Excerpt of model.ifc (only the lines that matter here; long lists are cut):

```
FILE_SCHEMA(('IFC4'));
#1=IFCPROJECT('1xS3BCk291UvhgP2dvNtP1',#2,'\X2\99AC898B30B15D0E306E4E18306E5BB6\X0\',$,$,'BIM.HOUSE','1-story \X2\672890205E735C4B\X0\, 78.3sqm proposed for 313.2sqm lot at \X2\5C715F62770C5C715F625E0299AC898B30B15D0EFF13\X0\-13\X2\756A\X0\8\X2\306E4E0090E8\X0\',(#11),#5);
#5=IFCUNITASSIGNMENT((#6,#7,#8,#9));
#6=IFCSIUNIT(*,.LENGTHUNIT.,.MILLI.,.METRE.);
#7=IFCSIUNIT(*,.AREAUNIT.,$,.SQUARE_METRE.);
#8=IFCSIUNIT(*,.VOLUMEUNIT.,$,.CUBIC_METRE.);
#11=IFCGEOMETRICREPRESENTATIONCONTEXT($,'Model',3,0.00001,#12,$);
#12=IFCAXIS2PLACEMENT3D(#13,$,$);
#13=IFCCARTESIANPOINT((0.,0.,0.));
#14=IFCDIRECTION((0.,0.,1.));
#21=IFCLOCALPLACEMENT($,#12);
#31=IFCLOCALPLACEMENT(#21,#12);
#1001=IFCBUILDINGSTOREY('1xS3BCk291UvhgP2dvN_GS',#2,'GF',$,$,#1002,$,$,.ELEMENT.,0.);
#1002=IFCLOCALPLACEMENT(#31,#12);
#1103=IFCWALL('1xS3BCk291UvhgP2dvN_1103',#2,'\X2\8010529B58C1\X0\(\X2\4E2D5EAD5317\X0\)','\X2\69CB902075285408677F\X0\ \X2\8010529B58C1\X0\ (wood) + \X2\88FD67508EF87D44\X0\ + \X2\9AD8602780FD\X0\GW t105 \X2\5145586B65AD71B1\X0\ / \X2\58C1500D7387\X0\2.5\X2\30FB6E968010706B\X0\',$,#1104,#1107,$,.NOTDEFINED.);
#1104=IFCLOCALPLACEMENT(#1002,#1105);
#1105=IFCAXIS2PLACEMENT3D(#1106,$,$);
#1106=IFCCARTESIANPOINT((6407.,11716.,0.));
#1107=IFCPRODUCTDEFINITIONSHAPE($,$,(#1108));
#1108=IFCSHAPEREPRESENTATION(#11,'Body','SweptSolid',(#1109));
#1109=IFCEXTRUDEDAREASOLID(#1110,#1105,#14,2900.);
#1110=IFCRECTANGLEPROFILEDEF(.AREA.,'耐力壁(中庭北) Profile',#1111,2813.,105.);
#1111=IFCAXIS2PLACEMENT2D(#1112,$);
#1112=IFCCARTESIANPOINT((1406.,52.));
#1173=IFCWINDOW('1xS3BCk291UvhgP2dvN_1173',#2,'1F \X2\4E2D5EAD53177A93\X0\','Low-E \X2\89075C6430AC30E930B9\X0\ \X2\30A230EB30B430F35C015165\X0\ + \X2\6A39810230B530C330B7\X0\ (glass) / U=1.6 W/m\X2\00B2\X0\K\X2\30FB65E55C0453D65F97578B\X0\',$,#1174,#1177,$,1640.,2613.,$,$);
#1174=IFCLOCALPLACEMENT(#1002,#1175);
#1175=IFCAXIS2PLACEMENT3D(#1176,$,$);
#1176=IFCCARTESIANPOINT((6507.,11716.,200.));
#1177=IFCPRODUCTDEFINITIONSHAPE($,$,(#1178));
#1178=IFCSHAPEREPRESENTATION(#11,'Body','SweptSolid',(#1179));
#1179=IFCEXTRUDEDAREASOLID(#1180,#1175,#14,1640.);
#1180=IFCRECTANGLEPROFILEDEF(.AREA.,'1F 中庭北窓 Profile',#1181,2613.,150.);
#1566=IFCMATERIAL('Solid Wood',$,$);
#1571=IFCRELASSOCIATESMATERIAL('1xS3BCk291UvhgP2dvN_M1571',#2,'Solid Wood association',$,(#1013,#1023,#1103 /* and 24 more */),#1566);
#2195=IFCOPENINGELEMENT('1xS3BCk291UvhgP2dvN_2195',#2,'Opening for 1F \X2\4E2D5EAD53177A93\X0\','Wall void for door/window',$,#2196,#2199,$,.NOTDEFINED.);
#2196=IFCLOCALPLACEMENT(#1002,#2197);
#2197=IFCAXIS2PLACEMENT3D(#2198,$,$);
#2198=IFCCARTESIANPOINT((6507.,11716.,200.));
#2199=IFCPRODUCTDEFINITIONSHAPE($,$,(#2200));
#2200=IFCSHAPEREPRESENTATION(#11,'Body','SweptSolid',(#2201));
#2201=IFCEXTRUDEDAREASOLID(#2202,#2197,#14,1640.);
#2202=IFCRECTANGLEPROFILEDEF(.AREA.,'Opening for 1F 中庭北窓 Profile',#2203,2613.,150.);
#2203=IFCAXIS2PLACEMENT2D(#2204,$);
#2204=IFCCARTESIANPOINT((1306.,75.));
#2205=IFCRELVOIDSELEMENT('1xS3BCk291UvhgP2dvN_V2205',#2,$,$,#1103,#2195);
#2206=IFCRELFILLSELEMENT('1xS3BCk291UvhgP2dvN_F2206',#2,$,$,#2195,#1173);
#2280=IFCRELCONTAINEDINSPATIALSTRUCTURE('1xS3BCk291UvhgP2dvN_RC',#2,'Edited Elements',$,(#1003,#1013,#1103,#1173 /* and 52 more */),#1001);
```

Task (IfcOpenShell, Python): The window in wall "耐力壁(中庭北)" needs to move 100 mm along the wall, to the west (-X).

```python
import ifcopenshell
import ifcopenshell.api.geometry
import ifcopenshell.util.placement
import ifcopenshell.util.unit

model = ifcopenshell.open("model.ifc")
unit_scale = ifcopenshell.util.unit.calculate_unit_scale(model)

window = model.by_guid("1xS3BCk291UvhgP2dvN_1173")
opening = window.FillsVoids[0].RelatingOpeningElement
wall = opening.VoidsElements[0].RelatingBuildingElement

wall_matrix = ifcopenshell.util.placement.get_local_placement(wall.ObjectPlacement)
shift = wall_matrix[:3, 0] * -0.1 / unit_scale
before = ifcopenshell.util.placement.get_local_placement(window.ObjectPlacement)[:3, 3].copy()

# The window is not placed relative to its opening, so move both.
for product in (opening, window):
    matrix = ifcopenshell.util.placement.get_local_placement(product.ObjectPlacement)
    matrix[:3, 3] += shift
    ifcopenshell.api.geometry.edit_object_placement(model, product=product, matrix=matrix, is_si=False)

after = ifcopenshell.util.placement.get_local_placement(window.ObjectPlacement)[:3, 3]
print("window moved by", (after - before).round(3) + 0.0)

model.write("model_rev.ifc")
```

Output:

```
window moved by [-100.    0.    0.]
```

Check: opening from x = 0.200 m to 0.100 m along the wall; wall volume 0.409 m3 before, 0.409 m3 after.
